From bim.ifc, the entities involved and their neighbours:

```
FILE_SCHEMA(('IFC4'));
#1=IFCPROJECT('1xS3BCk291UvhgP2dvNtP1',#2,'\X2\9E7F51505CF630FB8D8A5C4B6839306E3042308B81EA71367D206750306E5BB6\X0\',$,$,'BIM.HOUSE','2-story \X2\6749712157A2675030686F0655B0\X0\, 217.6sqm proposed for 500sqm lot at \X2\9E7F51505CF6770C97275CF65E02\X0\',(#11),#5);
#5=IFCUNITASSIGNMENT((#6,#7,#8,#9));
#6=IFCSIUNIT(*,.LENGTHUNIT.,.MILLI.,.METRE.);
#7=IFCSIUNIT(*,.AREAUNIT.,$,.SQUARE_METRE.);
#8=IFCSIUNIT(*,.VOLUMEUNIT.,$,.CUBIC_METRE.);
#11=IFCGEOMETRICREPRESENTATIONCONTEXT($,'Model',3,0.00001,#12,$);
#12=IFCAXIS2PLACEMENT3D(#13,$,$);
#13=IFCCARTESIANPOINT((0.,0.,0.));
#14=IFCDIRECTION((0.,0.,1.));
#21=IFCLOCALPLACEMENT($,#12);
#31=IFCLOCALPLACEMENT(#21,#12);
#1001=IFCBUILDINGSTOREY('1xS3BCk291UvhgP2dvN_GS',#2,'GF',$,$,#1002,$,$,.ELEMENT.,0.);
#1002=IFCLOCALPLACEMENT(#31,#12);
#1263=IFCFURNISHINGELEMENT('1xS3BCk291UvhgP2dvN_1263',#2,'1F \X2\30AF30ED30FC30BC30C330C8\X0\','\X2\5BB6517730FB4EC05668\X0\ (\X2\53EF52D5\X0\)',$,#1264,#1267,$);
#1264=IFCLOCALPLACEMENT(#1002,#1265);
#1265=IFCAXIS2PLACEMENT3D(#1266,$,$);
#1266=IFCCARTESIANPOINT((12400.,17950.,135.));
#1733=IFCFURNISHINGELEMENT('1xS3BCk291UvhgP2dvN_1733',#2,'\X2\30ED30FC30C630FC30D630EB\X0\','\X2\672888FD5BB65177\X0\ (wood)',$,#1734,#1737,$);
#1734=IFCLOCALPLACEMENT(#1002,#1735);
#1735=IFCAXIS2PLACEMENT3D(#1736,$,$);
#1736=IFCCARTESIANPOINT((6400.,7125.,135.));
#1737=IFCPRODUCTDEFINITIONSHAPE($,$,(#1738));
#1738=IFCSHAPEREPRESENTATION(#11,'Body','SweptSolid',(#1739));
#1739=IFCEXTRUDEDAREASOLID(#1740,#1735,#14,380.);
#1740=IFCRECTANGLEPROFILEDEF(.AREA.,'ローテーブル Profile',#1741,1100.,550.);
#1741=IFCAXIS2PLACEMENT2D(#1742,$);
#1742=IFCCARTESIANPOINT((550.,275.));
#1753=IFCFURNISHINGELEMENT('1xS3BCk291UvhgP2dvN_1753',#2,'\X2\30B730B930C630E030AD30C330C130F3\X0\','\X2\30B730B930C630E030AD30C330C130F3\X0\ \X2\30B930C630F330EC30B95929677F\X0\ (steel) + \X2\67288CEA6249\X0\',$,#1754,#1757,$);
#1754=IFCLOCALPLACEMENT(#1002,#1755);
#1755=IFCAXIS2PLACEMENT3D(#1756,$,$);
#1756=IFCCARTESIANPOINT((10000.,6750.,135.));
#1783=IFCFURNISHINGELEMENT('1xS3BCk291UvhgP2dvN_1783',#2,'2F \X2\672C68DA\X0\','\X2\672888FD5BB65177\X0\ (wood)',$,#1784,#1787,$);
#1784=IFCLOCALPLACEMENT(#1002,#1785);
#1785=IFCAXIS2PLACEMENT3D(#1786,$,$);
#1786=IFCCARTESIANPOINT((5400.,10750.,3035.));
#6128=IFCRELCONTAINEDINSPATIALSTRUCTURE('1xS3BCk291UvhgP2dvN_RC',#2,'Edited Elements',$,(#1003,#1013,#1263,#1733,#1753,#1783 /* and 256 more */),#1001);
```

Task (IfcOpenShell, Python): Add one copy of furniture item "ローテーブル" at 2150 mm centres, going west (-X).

```python
import numpy as np
import ifcopenshell
import ifcopenshell.api.geometry
import ifcopenshell.api.root
import ifcopenshell.util.element
import ifcopenshell.util.placement
import ifcopenshell.util.unit

model = ifcopenshell.open("bim.ifc")
unit_scale = ifcopenshell.util.unit.calculate_unit_scale(model)


def reuse_history(source, copy):
    """copy_class also copies each property set's owner history, people and application; keep the originals."""
    for rel in copy.IsDefinedBy:
        if rel.is_a("IfcRelDefinesByProperties") and (history := rel.RelatingPropertyDefinition.OwnerHistory):
            rel.RelatingPropertyDefinition.OwnerHistory = source.OwnerHistory
            ifcopenshell.util.element.remove_deep2(model, history)


source = model.by_id(1733)
base = ifcopenshell.util.placement.get_local_placement(source.ObjectPlacement)
step = np.array([-1.0, 0.0, 0.0]) * 2.15 / unit_scale

for i in range(1, 2):
    copy = ifcopenshell.api.root.copy_class(model, product=source)
    copy.Representation = ifcopenshell.util.element.copy_deep(
        model, source.Representation, exclude=["IfcGeometricRepresentationContext", "IfcRepresentationMap"]
    )
    reuse_history(source, copy)
    matrix = base.copy()
    matrix[:3, 3] += i * step
    print("added at", matrix[:3, 3].round(3) + 0.0)
    ifcopenshell.api.geometry.edit_object_placement(model, product=copy, matrix=matrix, is_si=False)

model.write("bim_edited.ifc")
```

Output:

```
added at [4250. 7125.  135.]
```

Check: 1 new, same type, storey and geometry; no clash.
